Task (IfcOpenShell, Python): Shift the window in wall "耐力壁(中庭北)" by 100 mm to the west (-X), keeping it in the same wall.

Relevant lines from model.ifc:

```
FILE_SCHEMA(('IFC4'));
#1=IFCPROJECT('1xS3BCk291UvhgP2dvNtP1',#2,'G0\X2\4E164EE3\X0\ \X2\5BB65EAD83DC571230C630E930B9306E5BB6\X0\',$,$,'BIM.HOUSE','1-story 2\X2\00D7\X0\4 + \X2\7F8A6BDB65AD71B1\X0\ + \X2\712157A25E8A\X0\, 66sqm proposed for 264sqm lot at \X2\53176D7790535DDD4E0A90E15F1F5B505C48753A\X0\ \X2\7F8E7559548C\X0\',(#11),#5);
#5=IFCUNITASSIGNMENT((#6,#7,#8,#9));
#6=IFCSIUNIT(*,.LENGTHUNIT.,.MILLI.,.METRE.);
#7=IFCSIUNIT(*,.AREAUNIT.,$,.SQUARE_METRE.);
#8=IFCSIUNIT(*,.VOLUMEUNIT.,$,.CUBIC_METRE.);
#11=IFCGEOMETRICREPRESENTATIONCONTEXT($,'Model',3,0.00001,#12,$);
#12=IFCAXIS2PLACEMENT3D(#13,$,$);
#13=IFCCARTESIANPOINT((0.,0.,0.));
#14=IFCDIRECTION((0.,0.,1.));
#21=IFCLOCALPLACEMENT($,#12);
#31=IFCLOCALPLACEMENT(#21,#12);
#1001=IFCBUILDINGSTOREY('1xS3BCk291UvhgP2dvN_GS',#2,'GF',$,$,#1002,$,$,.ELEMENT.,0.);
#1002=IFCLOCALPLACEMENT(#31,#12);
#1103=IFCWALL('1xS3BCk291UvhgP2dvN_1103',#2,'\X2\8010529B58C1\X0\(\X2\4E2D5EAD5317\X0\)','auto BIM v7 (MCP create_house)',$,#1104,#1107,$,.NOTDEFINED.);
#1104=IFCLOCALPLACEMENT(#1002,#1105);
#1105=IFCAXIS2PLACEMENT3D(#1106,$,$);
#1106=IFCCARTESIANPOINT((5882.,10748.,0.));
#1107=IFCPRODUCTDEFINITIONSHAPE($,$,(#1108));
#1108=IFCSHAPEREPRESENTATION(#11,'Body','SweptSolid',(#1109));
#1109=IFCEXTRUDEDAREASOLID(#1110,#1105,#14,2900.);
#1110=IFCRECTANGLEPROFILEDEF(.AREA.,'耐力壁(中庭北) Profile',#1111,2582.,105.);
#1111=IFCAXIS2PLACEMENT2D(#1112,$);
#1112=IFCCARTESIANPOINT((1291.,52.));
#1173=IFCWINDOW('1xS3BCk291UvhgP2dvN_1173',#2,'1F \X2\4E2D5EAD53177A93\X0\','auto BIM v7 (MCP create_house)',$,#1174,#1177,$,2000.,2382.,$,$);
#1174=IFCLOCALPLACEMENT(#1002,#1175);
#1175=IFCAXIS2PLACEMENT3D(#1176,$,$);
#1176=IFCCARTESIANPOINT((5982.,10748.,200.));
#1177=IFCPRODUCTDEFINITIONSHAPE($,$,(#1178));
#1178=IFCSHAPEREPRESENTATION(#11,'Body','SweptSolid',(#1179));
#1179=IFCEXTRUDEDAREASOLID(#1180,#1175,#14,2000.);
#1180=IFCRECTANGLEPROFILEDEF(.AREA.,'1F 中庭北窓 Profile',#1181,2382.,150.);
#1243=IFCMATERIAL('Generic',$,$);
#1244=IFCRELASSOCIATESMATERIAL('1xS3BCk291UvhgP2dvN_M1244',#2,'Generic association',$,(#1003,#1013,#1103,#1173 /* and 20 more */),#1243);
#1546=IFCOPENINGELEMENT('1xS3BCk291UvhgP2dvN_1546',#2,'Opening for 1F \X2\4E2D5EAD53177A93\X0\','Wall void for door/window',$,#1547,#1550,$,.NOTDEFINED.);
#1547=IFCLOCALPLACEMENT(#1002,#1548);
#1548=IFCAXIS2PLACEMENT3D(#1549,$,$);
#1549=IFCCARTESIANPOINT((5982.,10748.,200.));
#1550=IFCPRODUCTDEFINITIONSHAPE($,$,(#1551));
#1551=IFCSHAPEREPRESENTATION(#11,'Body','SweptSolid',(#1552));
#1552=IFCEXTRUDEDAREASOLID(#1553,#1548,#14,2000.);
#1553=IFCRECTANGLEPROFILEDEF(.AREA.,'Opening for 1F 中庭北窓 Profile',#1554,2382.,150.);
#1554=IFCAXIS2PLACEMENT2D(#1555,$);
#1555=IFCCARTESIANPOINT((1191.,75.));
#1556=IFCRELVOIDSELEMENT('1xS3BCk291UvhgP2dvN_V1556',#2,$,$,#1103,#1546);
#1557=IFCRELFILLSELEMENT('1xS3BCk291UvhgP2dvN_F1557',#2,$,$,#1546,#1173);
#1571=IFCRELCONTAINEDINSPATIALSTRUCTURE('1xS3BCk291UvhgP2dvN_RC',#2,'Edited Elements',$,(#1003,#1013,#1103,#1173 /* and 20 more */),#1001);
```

```python
import ifcopenshell
import ifcopenshell.api.geometry
import ifcopenshell.util.placement

model = ifcopenshell.open("model.ifc")

window = model.by_guid("1xS3BCk291UvhgP2dvN_1173")
opening = window.FillsVoids[0].RelatingOpeningElement
wall = opening.VoidsElements[0].RelatingBuildingElement

wall_matrix = ifcopenshell.util.placement.get_local_placement(wall.ObjectPlacement)
shift = wall_matrix[:3, 0] * -100.0
before = ifcopenshell.util.placement.get_local_placement(window.ObjectPlacement)[:3, 3].copy()

# The window is not placed relative to its opening, so move both.
for product in (opening, window):
    matrix = ifcopenshell.util.placement.get_local_placement(product.ObjectPlacement)
    matrix[:3, 3] += shift
    ifcopenshell.api.geometry.edit_object_placement(model, product=product, matrix=matrix, is_si=False)

after = ifcopenshell.util.placement.get_local_placement(window.ObjectPlacement)[:3, 3]
print("window moved by", (after - before).round(3) + 0.0)

model.write("model_updated.ifc")
```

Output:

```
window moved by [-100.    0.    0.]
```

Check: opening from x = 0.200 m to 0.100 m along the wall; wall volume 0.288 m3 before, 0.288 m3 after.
